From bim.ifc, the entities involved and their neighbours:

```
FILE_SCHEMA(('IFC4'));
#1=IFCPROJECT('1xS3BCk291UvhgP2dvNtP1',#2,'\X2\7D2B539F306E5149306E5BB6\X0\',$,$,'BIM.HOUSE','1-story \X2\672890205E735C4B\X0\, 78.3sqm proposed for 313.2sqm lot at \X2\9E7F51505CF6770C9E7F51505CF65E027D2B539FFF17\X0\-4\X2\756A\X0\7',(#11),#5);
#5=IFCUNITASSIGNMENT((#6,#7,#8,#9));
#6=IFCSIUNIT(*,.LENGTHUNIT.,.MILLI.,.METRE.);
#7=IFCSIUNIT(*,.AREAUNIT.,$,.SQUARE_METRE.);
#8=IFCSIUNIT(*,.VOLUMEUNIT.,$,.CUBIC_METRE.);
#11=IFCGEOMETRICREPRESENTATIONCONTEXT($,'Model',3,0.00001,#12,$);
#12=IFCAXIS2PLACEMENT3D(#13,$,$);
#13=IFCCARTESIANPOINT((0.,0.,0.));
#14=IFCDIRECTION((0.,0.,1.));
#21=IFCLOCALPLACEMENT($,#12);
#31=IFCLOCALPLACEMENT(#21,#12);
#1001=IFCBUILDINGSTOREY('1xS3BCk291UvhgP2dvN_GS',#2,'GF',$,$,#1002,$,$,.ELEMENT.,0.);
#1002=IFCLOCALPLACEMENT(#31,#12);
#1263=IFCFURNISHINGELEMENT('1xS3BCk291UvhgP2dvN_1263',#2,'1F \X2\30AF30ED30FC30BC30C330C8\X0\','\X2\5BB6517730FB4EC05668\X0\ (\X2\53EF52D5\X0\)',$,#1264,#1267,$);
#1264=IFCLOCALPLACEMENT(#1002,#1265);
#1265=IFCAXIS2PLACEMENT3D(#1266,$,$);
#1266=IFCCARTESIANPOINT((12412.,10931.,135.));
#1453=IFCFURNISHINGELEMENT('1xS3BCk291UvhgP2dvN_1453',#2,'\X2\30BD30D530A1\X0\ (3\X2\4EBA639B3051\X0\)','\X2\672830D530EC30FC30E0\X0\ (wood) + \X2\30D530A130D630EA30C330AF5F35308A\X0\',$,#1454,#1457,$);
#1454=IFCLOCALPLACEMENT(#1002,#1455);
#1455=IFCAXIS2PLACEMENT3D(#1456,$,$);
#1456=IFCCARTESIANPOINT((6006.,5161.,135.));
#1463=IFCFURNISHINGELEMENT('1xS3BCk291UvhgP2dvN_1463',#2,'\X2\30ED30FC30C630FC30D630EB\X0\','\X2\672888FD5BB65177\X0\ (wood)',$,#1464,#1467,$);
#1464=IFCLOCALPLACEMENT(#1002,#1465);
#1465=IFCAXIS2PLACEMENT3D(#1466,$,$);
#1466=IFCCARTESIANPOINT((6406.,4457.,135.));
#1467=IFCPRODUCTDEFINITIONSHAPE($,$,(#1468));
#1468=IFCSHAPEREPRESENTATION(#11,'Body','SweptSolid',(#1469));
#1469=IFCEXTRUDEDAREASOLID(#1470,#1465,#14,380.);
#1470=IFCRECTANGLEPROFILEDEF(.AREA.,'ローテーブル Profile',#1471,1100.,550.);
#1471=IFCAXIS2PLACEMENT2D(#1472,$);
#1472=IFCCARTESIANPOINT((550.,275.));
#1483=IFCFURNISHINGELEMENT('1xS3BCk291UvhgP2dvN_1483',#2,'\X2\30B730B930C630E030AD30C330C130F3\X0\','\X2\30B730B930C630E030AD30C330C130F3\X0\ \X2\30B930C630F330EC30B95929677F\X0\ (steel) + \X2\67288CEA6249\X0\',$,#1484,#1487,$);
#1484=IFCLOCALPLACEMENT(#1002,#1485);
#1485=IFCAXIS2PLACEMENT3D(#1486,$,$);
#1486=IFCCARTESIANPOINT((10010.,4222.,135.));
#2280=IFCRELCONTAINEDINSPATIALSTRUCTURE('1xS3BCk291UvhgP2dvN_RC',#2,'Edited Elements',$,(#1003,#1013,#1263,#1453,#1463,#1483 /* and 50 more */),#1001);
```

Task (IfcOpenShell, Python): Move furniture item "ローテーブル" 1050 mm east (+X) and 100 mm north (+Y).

```python
import ifcopenshell
import ifcopenshell.api.geometry
import ifcopenshell.util.placement
import ifcopenshell.util.unit

model = ifcopenshell.open("bim.ifc")
unit_scale = ifcopenshell.util.unit.calculate_unit_scale(model)

item = model.by_guid("1xS3BCk291UvhgP2dvN_1463")
matrix = ifcopenshell.util.placement.get_local_placement(item.ObjectPlacement)
matrix[0, 3] += 1.05 / unit_scale
matrix[1, 3] += 0.1 / unit_scale
ifcopenshell.api.geometry.edit_object_placement(model, product=item, matrix=matrix, is_si=False)

print(ifcopenshell.util.placement.get_local_placement(item.ObjectPlacement).round(3) + 0.0)

model.write("bim_edited.ifc")
```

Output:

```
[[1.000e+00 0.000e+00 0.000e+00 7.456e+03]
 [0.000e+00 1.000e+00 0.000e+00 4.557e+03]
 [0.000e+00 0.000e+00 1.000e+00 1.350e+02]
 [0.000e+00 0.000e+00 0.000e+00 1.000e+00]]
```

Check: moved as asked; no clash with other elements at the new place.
